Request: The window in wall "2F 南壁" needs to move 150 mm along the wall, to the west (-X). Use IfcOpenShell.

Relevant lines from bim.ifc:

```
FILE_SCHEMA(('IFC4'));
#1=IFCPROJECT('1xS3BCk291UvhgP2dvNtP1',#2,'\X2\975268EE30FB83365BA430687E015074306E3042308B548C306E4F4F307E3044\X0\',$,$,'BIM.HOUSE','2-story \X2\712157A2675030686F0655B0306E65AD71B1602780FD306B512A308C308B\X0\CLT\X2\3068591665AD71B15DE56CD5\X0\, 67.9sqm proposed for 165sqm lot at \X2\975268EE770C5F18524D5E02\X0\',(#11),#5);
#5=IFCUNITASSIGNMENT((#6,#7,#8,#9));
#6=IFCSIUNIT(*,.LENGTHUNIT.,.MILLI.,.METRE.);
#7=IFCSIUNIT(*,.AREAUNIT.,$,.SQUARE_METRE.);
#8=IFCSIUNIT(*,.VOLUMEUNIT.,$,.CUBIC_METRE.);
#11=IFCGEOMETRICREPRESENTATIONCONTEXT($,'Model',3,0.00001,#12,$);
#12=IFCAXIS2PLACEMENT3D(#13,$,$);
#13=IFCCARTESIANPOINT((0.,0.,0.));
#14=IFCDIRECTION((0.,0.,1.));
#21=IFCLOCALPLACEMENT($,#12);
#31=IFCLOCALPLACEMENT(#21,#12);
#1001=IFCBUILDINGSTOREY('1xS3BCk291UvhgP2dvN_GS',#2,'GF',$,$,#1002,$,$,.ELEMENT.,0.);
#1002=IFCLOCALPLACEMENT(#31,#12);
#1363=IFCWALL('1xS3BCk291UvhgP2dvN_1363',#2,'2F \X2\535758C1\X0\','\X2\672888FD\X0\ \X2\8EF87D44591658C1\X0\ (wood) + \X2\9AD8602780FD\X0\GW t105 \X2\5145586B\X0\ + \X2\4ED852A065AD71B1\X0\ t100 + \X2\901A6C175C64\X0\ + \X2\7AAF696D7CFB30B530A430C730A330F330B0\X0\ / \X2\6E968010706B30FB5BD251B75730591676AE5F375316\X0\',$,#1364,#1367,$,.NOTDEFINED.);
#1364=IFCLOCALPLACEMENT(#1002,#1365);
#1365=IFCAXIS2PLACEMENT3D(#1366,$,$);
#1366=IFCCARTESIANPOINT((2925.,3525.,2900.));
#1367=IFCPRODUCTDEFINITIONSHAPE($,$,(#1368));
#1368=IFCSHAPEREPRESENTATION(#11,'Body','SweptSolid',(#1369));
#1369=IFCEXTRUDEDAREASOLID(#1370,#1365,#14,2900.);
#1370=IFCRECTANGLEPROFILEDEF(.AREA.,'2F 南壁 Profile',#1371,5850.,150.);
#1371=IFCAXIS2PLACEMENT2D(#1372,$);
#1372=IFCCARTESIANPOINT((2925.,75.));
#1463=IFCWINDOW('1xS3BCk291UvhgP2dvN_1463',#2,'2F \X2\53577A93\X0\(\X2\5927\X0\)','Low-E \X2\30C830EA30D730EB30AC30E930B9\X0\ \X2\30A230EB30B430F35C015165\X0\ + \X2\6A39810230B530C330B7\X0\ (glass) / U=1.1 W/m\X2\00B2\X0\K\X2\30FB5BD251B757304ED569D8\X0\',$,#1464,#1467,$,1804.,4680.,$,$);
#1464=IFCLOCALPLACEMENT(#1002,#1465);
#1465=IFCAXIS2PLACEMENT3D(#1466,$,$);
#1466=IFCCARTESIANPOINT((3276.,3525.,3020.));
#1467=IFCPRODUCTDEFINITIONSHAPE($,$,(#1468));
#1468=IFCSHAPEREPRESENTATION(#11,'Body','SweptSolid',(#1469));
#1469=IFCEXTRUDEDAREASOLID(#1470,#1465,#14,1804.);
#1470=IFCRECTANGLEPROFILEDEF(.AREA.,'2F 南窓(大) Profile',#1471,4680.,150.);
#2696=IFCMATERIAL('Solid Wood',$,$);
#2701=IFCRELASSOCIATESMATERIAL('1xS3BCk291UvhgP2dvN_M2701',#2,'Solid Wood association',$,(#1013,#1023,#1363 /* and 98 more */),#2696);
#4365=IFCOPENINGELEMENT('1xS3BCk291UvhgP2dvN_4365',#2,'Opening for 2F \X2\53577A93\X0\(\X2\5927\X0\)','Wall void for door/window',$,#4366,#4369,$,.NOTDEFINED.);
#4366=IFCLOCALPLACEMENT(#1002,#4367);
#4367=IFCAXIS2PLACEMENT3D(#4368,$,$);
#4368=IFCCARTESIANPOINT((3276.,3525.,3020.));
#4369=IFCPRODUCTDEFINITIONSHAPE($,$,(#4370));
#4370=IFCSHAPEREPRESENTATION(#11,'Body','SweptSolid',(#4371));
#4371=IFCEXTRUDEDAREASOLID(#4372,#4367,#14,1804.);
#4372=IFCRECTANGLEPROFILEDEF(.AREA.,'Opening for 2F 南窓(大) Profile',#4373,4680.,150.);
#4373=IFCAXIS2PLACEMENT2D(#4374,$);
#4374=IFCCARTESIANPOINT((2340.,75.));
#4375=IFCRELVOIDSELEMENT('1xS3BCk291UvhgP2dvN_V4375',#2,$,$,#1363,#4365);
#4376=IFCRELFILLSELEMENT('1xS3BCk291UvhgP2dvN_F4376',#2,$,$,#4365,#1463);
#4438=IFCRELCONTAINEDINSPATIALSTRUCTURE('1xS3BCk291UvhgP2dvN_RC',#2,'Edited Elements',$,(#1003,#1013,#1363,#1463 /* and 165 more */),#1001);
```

```python
import ifcopenshell
import ifcopenshell.api.geometry
import ifcopenshell.util.placement
import ifcopenshell.util.unit

model = ifcopenshell.open("bim.ifc")
unit_scale = ifcopenshell.util.unit.calculate_unit_scale(model)

window = model.by_id(1463)
opening = window.FillsVoids[0].RelatingOpeningElement
wall = opening.VoidsElements[0].RelatingBuildingElement

wall_matrix = ifcopenshell.util.placement.get_local_placement(wall.ObjectPlacement)
shift = wall_matrix[:3, 0] * -0.15 / unit_scale
before = ifcopenshell.util.placement.get_local_placement(window.ObjectPlacement)[:3, 3].copy()

# The window is not placed relative to its opening, so move both.
for product in (opening, window):
    matrix = ifcopenshell.util.placement.get_local_placement(product.ObjectPlacement)
    matrix[:3, 3] += shift
    ifcopenshell.api.geometry.edit_object_placement(model, product=product, matrix=matrix, is_si=False)

after = ifcopenshell.util.placement.get_local_placement(window.ObjectPlacement)[:3, 3]
print("window moved by", (after - before).round(3) + 0.0)

model.write("bim_v2.ifc")
```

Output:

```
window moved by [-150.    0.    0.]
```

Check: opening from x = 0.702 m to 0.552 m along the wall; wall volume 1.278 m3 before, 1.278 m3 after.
